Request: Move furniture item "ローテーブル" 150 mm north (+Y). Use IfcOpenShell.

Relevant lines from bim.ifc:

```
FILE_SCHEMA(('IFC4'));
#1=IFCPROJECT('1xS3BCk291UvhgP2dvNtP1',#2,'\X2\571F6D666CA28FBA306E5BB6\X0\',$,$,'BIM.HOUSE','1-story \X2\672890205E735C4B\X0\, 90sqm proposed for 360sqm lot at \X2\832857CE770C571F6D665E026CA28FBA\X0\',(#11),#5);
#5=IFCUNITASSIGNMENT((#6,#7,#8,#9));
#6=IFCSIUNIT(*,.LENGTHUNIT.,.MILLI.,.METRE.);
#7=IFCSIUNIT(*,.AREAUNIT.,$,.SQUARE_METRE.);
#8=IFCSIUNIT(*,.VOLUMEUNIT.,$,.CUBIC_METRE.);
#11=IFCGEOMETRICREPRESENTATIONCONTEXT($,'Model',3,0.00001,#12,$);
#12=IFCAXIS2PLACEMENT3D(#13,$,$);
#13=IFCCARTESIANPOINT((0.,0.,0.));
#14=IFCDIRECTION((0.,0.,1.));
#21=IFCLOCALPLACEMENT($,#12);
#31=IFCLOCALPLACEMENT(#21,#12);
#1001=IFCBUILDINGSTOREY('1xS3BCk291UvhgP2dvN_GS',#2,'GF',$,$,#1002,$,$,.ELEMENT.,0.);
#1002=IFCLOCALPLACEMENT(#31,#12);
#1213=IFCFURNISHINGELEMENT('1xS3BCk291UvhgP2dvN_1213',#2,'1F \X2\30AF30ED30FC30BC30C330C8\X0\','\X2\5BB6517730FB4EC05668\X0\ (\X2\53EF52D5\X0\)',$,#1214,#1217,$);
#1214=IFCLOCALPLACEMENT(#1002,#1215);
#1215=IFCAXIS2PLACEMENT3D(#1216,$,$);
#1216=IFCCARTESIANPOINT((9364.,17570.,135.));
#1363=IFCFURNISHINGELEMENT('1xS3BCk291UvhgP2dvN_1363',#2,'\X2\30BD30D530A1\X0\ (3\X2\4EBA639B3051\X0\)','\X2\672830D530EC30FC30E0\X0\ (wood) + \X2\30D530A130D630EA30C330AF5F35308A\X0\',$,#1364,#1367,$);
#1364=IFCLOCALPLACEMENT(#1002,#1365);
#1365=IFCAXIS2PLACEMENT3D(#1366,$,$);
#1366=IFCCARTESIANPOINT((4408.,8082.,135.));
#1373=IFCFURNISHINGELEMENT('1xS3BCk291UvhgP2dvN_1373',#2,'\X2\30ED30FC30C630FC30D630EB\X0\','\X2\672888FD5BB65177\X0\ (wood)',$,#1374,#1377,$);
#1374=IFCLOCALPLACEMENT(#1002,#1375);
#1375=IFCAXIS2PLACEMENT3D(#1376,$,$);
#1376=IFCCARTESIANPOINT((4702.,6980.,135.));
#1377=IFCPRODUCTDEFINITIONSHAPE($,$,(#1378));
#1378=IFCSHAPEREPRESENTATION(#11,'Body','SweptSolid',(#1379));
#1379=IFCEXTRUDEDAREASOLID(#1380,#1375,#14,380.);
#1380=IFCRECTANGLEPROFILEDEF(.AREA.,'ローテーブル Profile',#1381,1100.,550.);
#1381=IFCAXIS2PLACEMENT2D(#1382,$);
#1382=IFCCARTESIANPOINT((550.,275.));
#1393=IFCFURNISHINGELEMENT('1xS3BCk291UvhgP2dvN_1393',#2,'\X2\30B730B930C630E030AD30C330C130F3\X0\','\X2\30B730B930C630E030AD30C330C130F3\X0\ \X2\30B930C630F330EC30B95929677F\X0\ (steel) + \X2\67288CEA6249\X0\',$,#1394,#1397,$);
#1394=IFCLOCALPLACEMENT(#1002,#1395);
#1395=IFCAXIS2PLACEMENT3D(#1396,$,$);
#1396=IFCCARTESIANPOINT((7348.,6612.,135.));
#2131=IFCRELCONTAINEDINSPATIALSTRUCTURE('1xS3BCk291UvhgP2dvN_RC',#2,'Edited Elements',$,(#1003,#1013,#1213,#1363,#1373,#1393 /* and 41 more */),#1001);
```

```python
import ifcopenshell
import ifcopenshell.api.geometry
import ifcopenshell.util.placement

model = ifcopenshell.open("bim.ifc")

item = model.by_id(1373)
matrix = ifcopenshell.util.placement.get_local_placement(item.ObjectPlacement)
matrix[1, 3] += 150.0
ifcopenshell.api.geometry.edit_object_placement(model, product=item, matrix=matrix, is_si=False)

print(ifcopenshell.util.placement.get_local_placement(item.ObjectPlacement).round(3) + 0.0)

model.write("bim_v2.ifc")
```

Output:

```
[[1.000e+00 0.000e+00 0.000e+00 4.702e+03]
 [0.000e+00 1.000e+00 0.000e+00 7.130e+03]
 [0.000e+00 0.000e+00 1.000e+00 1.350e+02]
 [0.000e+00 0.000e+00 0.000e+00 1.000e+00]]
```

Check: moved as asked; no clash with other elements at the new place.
